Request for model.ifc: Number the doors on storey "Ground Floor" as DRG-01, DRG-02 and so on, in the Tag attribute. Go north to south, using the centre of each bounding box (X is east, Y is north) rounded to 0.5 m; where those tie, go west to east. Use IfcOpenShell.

First a look at what the model holds.

```python
import ifcopenshell
import ifcopenshell.util.element
import ifcopenshell.util.placement

model = ifcopenshell.open("model.ifc")
print(model.schema)
storey = next(s for s in model.by_type("IfcBuildingStorey") if s.Name == "Ground Floor")
doors = [e for e in ifcopenshell.util.element.get_decomposition(storey) if e.is_a("IfcDoor")]
for e in sorted(doors, key=lambda e: e.id()):
    origin = ifcopenshell.util.placement.get_local_placement(e.ObjectPlacement)[:3, 3]
    print(e.id(), e.Tag, e.Name, origin.round(2) + 0.0, sep=" | ")
```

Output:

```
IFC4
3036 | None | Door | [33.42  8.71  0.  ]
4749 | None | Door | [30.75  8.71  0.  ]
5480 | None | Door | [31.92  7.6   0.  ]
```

```python
import ifcopenshell
import ifcopenshell.geom
import ifcopenshell.util.element
import ifcopenshell.util.shape

model = ifcopenshell.open("model.ifc")
settings = ifcopenshell.geom.settings()
settings.set("use-world-coords", True)


def centre(element):
    shape = ifcopenshell.geom.create_shape(settings, element)
    return ifcopenshell.util.shape.get_bbox_centroid(shape.geometry)


storey = next(s for s in model.by_type("IfcBuildingStorey") if s.Name == "Ground Floor")
doors = [e for e in ifcopenshell.util.element.get_decomposition(storey) if e.is_a("IfcDoor")]

# Insertion points can sit at a corner or the storey origin, so sort by the geometry (in metres).
centres = {e: centre(e) for e in doors}
doors.sort(key=lambda e: (-round(centres[e][1] / 0.5), centres[e][0]))

for i, e in enumerate(doors, start=1):
    number = f"DRG-{i:02d}"
    e.Tag = number
    print(e.id(), number)

model.write("model_updated.ifc")
```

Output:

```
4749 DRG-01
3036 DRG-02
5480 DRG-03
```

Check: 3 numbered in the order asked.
